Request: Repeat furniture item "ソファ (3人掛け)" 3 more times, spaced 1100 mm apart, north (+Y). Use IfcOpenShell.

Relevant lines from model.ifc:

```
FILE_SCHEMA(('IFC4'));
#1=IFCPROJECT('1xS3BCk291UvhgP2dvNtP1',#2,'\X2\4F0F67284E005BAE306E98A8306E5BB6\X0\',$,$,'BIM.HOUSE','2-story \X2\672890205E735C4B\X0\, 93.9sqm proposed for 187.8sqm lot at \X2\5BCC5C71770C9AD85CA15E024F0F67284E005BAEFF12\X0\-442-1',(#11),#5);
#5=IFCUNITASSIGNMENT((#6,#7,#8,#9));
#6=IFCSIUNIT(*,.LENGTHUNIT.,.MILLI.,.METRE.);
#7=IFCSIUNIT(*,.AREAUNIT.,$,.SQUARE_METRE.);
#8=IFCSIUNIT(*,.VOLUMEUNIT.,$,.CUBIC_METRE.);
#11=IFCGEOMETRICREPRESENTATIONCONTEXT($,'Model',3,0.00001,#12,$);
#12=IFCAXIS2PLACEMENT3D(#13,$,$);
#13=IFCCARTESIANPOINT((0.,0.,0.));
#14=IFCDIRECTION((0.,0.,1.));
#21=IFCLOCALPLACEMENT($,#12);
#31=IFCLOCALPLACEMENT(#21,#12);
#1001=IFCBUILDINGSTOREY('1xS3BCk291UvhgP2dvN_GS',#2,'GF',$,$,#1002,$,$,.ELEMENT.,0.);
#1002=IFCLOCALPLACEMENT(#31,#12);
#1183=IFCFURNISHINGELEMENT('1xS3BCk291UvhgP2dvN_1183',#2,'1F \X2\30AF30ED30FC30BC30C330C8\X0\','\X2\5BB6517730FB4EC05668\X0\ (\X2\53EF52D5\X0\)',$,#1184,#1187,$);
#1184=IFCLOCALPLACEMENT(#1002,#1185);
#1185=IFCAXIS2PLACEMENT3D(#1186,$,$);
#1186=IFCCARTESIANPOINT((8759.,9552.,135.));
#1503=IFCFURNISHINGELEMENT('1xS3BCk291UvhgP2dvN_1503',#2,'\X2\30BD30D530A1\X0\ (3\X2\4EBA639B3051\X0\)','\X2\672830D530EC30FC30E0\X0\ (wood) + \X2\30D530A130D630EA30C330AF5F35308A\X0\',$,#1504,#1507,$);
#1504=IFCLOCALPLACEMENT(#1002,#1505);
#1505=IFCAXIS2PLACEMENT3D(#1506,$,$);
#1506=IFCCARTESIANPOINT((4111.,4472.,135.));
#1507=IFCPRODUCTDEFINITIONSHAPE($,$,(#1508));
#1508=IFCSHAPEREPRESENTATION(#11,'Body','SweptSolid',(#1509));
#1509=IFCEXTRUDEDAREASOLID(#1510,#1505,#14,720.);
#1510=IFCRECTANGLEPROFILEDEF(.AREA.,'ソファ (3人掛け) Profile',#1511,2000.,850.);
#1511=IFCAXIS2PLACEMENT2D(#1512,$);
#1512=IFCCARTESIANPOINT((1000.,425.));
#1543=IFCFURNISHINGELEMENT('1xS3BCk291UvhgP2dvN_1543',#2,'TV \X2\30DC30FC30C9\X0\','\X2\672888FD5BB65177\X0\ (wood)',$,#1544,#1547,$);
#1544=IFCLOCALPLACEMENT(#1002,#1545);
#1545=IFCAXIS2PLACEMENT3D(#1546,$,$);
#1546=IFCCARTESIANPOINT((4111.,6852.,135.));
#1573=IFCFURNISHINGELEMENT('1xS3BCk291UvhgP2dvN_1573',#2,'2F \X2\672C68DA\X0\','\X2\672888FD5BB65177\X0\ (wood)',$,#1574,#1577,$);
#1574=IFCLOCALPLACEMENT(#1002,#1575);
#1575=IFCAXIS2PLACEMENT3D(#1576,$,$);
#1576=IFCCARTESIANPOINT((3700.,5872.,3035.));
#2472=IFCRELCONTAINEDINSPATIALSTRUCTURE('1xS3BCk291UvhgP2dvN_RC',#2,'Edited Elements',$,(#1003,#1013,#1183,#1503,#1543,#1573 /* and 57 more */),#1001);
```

```python
import numpy as np
import ifcopenshell
import ifcopenshell.api.geometry
import ifcopenshell.api.root
import ifcopenshell.util.element
import ifcopenshell.util.placement

model = ifcopenshell.open("model.ifc")


def reuse_history(source, copy):
    """copy_class also copies each property set's owner history, people and application; keep the originals."""
    for rel in copy.IsDefinedBy:
        if rel.is_a("IfcRelDefinesByProperties") and (history := rel.RelatingPropertyDefinition.OwnerHistory):
            rel.RelatingPropertyDefinition.OwnerHistory = source.OwnerHistory
            ifcopenshell.util.element.remove_deep2(model, history)


source = model.by_id(1503)
base = ifcopenshell.util.placement.get_local_placement(source.ObjectPlacement)
step = np.array([0.0, 1.0, 0.0]) * 1100.0

for i in range(1, 4):
    copy = ifcopenshell.api.root.copy_class(model, product=source)
    copy.Representation = ifcopenshell.util.element.copy_deep(
        model, source.Representation, exclude=["IfcGeometricRepresentationContext", "IfcRepresentationMap"]
    )
    reuse_history(source, copy)
    matrix = base.copy()
    matrix[:3, 3] += i * step
    print("added at", matrix[:3, 3].round(3) + 0.0)
    ifcopenshell.api.geometry.edit_object_placement(model, product=copy, matrix=matrix, is_si=False)

model.write("model-out.ifc")
```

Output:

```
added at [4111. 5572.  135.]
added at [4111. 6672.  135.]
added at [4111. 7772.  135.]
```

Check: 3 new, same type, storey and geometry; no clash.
